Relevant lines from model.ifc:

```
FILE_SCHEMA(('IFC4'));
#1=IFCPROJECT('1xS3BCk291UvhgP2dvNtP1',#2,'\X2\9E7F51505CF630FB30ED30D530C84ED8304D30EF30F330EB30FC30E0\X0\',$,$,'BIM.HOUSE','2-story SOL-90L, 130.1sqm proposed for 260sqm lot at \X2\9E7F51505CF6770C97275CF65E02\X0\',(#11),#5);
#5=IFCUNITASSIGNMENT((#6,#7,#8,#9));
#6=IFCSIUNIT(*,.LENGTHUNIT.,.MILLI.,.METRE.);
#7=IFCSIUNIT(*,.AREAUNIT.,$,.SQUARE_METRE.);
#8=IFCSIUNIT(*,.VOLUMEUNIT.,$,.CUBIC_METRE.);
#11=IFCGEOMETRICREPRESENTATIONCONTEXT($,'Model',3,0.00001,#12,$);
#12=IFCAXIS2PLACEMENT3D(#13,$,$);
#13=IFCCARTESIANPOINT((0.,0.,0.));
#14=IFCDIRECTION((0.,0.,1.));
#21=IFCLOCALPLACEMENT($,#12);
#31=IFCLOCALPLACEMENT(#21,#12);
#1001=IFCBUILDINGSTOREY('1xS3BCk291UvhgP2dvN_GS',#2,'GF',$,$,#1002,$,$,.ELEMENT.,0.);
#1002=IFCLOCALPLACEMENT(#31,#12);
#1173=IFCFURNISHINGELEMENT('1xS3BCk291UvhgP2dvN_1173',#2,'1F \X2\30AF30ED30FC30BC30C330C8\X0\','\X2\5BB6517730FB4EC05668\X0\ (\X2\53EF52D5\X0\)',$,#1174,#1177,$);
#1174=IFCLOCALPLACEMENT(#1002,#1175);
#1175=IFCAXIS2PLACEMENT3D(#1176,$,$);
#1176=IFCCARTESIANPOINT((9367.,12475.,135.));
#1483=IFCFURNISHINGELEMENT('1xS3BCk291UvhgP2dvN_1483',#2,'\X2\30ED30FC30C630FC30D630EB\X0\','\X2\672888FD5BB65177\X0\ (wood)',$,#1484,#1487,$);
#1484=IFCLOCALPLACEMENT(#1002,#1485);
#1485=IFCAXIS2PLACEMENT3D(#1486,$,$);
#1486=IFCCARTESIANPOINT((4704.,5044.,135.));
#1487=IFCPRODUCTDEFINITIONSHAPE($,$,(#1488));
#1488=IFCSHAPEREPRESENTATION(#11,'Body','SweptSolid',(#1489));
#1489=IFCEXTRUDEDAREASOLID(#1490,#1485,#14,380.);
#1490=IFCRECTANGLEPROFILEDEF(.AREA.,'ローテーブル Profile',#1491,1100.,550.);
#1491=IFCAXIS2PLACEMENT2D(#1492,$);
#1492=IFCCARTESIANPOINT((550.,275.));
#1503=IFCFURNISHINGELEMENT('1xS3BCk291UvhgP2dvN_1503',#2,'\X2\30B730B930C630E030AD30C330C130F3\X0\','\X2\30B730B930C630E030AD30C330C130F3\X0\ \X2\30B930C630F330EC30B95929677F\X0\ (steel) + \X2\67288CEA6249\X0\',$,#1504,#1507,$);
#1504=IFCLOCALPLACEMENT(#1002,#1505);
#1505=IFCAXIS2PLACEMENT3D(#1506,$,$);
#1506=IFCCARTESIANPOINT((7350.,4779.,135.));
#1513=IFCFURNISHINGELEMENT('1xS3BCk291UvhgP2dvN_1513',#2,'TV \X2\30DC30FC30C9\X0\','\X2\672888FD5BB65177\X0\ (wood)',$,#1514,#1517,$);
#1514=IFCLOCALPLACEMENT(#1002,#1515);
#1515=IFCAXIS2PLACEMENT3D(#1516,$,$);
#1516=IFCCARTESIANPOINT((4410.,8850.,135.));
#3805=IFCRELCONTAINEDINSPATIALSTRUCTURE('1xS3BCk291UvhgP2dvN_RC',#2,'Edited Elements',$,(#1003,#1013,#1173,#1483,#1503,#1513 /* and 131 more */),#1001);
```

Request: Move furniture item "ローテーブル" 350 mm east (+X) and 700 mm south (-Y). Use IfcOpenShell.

```python
import ifcopenshell
import ifcopenshell.api.geometry
import ifcopenshell.util.placement
import ifcopenshell.util.unit

model = ifcopenshell.open("model.ifc")
unit_scale = ifcopenshell.util.unit.calculate_unit_scale(model)

item = model.by_id(1483)
matrix = ifcopenshell.util.placement.get_local_placement(item.ObjectPlacement)
matrix[0, 3] += 0.35 / unit_scale
matrix[1, 3] -= 0.7 / unit_scale
ifcopenshell.api.geometry.edit_object_placement(model, product=item, matrix=matrix, is_si=False)

print(ifcopenshell.util.placement.get_local_placement(item.ObjectPlacement).round(3) + 0.0)

model.write("model_v2.ifc")
```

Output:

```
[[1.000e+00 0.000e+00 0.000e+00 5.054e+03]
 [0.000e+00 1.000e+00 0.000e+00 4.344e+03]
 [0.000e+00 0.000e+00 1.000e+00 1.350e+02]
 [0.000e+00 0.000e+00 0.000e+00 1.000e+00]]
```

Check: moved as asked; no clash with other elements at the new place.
